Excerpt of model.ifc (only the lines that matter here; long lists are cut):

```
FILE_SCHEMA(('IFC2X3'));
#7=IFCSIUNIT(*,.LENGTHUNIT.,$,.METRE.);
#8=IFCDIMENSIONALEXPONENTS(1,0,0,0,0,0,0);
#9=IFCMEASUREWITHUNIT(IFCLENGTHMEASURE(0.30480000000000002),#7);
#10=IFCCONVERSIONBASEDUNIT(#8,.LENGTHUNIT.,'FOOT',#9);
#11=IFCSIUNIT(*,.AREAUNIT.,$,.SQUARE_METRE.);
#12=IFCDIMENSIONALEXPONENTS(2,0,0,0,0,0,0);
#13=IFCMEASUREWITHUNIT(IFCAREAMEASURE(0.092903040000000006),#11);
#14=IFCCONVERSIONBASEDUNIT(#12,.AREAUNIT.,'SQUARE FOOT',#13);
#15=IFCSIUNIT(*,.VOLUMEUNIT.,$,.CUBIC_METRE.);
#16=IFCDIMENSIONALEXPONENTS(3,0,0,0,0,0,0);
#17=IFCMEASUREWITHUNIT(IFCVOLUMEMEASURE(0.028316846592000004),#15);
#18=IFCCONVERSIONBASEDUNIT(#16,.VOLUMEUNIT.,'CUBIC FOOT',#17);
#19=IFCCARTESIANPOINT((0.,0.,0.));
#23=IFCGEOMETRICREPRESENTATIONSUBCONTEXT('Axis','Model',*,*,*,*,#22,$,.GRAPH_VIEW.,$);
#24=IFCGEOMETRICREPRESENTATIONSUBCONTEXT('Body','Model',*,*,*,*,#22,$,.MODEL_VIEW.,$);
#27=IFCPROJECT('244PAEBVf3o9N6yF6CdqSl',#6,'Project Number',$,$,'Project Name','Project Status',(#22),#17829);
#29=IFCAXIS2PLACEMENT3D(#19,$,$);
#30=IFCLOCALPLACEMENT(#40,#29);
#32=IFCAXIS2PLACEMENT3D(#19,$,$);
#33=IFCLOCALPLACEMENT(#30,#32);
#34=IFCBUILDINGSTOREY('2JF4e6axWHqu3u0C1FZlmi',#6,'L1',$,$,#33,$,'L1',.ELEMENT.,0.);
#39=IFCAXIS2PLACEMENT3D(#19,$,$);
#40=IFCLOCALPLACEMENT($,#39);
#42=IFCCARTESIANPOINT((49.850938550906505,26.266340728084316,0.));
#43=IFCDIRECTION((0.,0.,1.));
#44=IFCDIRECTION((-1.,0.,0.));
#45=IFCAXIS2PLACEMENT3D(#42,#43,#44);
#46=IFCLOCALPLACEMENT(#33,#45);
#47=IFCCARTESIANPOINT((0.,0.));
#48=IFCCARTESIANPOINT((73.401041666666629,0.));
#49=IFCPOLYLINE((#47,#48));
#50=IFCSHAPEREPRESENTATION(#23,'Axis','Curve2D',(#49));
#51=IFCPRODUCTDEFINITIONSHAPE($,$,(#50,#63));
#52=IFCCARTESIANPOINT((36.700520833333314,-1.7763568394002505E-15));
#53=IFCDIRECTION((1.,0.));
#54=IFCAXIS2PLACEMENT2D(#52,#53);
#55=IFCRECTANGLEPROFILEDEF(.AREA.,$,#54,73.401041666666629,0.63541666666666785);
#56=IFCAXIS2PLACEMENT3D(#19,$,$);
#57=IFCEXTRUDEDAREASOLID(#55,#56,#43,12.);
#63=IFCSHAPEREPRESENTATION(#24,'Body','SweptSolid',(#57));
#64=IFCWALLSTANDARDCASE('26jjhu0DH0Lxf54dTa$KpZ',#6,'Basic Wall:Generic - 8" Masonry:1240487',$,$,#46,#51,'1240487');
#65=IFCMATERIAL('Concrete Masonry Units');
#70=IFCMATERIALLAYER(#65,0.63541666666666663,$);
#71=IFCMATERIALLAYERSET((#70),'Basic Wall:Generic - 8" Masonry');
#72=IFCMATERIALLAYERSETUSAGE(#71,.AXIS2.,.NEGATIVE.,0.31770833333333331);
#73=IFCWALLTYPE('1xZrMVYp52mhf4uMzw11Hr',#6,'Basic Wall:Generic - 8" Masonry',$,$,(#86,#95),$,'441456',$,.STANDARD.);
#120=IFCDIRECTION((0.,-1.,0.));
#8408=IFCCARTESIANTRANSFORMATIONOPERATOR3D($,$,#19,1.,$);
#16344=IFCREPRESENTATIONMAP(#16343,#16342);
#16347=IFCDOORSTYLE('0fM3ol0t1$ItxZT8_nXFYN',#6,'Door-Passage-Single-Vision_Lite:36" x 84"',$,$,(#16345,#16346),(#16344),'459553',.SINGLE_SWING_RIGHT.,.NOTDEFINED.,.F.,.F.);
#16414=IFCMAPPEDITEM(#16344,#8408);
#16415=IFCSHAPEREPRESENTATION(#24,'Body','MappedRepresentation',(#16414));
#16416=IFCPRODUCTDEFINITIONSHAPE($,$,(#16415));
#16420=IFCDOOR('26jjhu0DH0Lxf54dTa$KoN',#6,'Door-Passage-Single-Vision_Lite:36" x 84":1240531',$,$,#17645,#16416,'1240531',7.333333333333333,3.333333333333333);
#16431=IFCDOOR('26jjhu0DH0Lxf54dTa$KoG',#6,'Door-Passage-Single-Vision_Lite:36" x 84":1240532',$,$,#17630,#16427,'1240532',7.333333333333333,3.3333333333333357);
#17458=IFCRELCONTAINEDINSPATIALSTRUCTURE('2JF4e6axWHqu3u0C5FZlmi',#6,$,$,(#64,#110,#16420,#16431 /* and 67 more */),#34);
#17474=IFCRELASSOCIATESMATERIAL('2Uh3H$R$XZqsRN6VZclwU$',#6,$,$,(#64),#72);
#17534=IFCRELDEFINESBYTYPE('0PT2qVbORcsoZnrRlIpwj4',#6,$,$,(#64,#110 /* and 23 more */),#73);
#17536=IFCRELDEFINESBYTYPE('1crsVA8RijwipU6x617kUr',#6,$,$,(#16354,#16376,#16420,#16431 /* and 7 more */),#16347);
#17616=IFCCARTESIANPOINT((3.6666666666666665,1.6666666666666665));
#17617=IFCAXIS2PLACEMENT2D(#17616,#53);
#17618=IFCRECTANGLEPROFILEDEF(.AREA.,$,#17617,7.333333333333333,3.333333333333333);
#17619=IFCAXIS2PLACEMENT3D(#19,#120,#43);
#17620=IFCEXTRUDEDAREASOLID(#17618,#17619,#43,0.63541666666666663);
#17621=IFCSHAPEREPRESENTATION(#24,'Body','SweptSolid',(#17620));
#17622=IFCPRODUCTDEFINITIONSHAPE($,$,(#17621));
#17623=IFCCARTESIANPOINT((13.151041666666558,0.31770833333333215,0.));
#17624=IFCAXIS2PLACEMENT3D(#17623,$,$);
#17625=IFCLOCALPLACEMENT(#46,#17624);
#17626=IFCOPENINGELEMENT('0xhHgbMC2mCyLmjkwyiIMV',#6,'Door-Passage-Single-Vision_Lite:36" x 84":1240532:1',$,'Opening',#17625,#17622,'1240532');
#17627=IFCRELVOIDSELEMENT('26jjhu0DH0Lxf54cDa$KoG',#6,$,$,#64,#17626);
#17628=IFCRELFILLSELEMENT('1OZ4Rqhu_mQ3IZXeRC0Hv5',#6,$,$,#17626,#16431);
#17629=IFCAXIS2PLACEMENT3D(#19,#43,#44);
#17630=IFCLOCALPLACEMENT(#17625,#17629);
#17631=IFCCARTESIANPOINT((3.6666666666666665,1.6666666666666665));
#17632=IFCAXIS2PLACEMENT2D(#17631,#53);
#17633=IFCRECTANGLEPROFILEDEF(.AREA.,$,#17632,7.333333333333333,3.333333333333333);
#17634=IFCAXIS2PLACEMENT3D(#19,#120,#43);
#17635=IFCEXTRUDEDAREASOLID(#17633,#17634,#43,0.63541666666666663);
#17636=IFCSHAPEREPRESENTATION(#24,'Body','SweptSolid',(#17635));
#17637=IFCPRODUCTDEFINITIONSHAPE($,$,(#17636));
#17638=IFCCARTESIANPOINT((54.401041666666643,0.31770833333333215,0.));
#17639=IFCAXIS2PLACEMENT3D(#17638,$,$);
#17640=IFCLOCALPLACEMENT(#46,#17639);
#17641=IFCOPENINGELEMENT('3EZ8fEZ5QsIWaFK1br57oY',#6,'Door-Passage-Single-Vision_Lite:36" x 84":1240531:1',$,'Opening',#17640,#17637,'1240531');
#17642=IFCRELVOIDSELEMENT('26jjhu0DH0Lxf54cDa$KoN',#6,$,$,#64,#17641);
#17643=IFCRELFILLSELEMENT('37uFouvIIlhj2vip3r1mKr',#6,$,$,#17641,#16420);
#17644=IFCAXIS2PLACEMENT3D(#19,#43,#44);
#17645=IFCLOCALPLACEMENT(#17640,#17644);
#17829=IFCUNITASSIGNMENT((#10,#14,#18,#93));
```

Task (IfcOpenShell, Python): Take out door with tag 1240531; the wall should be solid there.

```python
import ifcopenshell
import ifcopenshell.api.feature
import ifcopenshell.api.root
import ifcopenshell.geom
import ifcopenshell.util.shape

model = ifcopenshell.open("model.ifc")
settings = ifcopenshell.geom.settings()


def volume(element):
    """Net volume in cubic metres, openings subtracted."""
    shape = ifcopenshell.geom.create_shape(settings, element)
    return ifcopenshell.util.shape.get_volume(shape.geometry)


door = model.by_guid("26jjhu0DH0Lxf54dTa$KoN")
opening = door.FillsVoids[0].RelatingOpeningElement
wall = opening.VoidsElements[0].RelatingBuildingElement
before = volume(wall)

ifcopenshell.api.root.remove_product(model, product=door)
ifcopenshell.api.feature.remove_feature(model, feature=opening)

after = volume(wall)

print(f"wall volume {before:.3f} -> {after:.3f} m3")

model.write("model_updated.ifc")
```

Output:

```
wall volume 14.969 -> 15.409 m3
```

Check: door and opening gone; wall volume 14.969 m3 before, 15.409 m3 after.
